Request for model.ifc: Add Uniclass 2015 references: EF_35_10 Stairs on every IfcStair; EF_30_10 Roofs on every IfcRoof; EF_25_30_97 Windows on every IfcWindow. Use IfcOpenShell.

First a look at what the model holds.

```python
import ifcopenshell

model = ifcopenshell.open("model.ifc")
print(model.schema)
print("classifications:", [c.Name for c in model.by_type("IfcClassification")])
for ifc_class in ("IfcDoor", "IfcRoof", "IfcStair", "IfcWall", "IfcWindow"):
    print(ifc_class, len(model.by_type(ifc_class)))
```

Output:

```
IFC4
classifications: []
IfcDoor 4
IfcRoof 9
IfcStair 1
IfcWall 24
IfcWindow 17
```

```python
import ifcopenshell
import ifcopenshell.api.classification

model = ifcopenshell.open("model.ifc")

system = ifcopenshell.api.classification.add_classification(model, classification="Uniclass 2015")

codes = {
    "IfcStair": ("EF_35_10", "Stairs"),
    "IfcRoof": ("EF_30_10", "Roofs"),
    "IfcWindow": ("EF_25_30_97", "Windows"),
}
for ifc_class, (code, name) in codes.items():
    products = model.by_type(ifc_class)
    ifcopenshell.api.classification.add_reference(
        model, products=products, classification=system, identification=code, name=name
    )
    print(code, len(products))

model.write("model_v2.ifc")
```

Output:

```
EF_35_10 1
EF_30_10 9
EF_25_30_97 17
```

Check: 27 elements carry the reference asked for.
